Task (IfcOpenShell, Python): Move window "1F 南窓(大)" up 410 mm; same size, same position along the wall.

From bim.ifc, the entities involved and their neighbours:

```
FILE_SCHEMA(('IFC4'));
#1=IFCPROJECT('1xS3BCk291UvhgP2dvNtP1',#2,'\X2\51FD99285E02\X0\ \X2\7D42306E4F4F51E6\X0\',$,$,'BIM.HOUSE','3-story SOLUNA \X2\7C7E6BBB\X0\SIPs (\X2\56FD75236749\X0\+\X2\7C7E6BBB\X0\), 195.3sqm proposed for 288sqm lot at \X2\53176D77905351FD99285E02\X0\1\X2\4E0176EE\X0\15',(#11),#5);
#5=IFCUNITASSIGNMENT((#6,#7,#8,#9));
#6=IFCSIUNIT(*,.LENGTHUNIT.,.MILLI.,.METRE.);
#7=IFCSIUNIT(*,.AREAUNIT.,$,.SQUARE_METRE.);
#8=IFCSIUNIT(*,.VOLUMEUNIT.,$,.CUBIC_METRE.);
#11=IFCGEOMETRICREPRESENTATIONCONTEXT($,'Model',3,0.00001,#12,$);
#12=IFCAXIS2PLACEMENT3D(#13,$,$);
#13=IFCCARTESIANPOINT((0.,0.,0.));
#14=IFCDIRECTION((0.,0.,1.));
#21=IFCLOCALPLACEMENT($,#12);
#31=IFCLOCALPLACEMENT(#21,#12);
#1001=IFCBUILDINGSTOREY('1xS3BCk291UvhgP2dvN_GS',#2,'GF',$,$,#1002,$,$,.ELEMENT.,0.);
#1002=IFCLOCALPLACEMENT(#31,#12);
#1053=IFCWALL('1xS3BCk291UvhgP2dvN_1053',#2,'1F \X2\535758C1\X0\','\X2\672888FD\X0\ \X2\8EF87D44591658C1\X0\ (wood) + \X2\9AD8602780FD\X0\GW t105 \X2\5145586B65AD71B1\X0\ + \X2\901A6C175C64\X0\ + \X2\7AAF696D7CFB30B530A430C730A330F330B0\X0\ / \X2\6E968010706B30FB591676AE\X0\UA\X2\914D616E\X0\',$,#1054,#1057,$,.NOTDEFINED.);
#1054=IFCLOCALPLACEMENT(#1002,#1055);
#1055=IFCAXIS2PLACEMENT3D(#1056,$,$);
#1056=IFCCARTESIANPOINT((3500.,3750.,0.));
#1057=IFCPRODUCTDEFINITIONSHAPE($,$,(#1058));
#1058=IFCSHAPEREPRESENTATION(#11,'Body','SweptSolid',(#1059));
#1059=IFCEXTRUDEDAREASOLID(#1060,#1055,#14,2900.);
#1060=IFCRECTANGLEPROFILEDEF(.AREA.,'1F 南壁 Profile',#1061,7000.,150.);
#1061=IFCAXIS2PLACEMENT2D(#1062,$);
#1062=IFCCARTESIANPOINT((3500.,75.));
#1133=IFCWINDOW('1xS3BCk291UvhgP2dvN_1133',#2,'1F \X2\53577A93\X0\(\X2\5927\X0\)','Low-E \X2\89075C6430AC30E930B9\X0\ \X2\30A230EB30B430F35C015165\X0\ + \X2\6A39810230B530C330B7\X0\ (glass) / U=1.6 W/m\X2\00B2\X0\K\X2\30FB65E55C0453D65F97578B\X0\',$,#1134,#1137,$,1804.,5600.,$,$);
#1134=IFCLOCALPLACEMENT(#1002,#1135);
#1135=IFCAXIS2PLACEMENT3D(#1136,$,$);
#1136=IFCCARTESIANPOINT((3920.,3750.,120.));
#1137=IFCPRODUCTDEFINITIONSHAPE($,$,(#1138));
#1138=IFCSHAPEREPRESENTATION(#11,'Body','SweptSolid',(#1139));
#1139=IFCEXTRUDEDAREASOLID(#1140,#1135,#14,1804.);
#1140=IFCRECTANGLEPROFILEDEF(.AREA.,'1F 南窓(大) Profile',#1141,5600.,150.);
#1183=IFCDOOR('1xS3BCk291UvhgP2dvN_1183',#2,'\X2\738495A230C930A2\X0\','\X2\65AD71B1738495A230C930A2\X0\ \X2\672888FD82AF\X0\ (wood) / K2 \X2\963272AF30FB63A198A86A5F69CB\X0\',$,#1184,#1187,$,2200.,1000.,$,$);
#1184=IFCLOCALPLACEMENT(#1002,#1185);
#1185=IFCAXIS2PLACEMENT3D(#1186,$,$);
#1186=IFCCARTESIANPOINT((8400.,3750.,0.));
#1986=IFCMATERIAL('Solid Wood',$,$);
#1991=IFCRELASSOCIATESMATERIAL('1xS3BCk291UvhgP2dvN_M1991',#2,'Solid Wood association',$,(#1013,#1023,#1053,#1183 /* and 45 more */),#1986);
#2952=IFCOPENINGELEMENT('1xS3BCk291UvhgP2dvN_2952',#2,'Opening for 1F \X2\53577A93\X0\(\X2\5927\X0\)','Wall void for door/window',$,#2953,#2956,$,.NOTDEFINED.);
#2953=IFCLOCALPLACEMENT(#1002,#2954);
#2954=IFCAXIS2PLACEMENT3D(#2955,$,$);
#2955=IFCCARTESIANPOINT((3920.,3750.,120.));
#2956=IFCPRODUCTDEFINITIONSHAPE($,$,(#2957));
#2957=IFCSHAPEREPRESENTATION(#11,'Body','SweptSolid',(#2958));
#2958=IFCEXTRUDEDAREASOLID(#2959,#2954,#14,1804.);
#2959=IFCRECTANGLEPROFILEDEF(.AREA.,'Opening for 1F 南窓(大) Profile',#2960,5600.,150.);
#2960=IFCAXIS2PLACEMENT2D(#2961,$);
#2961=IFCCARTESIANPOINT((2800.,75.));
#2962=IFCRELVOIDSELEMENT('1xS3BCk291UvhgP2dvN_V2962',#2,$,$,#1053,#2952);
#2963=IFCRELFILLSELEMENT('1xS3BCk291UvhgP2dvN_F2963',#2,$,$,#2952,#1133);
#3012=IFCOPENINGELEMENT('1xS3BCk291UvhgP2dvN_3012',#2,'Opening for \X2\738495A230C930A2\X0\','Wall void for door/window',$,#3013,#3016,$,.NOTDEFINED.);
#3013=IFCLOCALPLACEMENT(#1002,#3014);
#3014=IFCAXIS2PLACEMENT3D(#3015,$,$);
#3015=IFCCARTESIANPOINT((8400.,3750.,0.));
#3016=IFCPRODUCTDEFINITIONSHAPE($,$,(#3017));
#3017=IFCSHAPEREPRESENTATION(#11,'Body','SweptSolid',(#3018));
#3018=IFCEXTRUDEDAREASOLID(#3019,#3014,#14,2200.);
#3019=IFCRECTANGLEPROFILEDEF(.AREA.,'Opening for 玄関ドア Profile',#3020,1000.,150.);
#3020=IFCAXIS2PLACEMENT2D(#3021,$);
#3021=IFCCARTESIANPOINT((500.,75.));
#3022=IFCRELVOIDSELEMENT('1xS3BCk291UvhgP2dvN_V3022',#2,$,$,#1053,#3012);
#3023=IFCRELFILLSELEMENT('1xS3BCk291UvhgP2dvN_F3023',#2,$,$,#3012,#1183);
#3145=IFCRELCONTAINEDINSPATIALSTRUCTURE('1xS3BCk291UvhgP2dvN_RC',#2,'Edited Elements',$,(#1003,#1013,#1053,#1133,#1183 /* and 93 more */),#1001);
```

```python
import numpy as np
import ifcopenshell
import ifcopenshell.api.geometry
import ifcopenshell.util.placement
import ifcopenshell.util.unit

model = ifcopenshell.open("bim.ifc")
unit_scale = ifcopenshell.util.unit.calculate_unit_scale(model)

window = model.by_guid("1xS3BCk291UvhgP2dvN_1133")
opening = window.FillsVoids[0].RelatingOpeningElement
dz = 410.0

shift = np.array([0.0, 0.0, dz])
# The window is not placed relative to its opening, so move both.
for product in (opening, window):
    matrix = ifcopenshell.util.placement.get_local_placement(product.ObjectPlacement)
    matrix[:3, 3] += shift
    ifcopenshell.api.geometry.edit_object_placement(model, product=product, matrix=matrix, is_si=False)

print(f"moved by {dz * unit_scale:+.3f} m")

model.write("bim_updated.ifc")
```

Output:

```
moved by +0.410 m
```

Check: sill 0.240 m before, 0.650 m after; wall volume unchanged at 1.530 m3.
